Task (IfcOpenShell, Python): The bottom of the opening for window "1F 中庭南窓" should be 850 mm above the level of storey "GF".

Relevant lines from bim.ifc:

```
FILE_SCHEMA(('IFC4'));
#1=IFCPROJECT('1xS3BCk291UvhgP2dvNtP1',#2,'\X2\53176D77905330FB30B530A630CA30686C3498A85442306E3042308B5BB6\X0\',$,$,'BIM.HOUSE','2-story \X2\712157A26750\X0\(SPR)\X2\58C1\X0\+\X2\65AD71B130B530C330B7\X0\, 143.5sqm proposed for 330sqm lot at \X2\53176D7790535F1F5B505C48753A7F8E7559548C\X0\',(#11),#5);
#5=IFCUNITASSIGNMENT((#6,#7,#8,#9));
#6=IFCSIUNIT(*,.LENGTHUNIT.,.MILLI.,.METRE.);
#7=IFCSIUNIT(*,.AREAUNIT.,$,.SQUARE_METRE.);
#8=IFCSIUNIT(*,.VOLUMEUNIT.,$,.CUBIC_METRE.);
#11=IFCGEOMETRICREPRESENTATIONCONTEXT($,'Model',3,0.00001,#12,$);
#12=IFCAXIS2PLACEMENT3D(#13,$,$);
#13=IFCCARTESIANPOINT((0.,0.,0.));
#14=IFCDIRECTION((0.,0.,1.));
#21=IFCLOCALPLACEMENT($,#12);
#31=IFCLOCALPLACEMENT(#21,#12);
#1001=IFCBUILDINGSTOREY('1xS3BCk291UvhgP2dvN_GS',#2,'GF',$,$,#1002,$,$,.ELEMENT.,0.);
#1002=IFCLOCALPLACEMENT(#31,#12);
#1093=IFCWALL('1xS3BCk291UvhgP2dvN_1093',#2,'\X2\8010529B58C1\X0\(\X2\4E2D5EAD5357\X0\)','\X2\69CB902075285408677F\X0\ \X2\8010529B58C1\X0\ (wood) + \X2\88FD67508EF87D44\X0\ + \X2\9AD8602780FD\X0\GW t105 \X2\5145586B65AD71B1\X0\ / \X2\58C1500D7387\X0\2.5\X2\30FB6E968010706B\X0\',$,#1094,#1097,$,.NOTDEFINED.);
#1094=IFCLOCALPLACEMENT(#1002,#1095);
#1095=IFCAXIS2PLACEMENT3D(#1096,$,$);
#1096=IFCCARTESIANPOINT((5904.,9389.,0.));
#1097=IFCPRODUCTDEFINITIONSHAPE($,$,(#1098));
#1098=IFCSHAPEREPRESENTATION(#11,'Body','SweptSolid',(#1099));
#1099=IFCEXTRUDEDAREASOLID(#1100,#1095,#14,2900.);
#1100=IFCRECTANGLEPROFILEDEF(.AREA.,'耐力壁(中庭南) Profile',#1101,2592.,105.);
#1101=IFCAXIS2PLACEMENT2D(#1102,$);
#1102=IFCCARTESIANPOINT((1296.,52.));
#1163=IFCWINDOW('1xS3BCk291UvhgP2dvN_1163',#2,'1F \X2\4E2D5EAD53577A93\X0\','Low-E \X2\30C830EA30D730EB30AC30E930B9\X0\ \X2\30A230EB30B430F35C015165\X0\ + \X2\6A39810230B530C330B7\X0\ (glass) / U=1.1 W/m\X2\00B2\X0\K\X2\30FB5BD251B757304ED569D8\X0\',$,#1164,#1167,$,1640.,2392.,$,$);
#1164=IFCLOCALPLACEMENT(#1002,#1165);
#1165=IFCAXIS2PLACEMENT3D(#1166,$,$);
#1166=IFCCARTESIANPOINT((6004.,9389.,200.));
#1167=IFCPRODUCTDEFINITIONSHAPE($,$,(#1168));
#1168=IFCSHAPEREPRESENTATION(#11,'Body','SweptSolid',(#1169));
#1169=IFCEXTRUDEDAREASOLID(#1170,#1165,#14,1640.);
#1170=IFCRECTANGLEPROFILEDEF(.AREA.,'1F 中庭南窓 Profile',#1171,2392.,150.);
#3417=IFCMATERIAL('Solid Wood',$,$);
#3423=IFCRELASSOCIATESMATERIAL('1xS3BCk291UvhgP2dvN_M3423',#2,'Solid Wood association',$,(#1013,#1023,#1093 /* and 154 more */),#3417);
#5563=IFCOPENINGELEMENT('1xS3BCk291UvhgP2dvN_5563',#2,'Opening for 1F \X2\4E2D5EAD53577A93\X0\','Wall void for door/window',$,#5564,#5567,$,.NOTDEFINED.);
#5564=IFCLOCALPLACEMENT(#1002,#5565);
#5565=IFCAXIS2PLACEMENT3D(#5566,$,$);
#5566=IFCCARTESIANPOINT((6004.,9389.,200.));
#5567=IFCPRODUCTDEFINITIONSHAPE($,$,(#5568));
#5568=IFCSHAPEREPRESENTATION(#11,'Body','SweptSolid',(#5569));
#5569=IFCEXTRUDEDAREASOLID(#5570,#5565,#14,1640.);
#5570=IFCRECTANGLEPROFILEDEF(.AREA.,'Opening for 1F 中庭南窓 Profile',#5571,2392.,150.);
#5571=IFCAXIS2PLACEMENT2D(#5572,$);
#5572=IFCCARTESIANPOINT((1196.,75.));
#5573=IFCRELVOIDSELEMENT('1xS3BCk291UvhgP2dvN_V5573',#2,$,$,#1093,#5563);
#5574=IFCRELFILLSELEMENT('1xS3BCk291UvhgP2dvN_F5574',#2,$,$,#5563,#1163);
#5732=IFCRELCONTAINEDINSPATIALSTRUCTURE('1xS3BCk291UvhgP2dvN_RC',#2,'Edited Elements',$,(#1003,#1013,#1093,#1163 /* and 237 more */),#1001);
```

```python
import numpy as np
import ifcopenshell
import ifcopenshell.api.geometry
import ifcopenshell.geom
import ifcopenshell.util.element
import ifcopenshell.util.placement
import ifcopenshell.util.shape
import ifcopenshell.util.unit

model = ifcopenshell.open("bim.ifc")
unit_scale = ifcopenshell.util.unit.calculate_unit_scale(model)

window = model.by_id(1163)
opening = window.FillsVoids[0].RelatingOpeningElement
storey = ifcopenshell.util.element.get_container(window, ifc_class="IfcBuildingStorey")
level = ifcopenshell.util.placement.get_local_placement(storey.ObjectPlacement)[2, 3]

# The opening's origin need not be at the sill, so measure its lowest point.
shape = ifcopenshell.geom.create_shape(ifcopenshell.geom.settings(), opening)
bottom = ifcopenshell.util.shape.get_shape_bottom_elevation(shape, shape.geometry) / unit_scale
dz = level + 850.0 - bottom

shift = np.array([0.0, 0.0, dz])
# The window is not placed relative to its opening, so move both.
for product in (opening, window):
    matrix = ifcopenshell.util.placement.get_local_placement(product.ObjectPlacement)
    matrix[:3, 3] += shift
    ifcopenshell.api.geometry.edit_object_placement(model, product=product, matrix=matrix, is_si=False)

print(f"moved by {dz * unit_scale:+.3f} m")

model.write("bim-out.ifc")
```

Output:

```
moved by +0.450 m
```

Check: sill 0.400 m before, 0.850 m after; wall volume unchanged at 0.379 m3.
